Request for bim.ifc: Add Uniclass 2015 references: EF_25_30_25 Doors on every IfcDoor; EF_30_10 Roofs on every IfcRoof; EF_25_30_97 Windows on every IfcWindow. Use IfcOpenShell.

First a look at what the model holds.

```python
import ifcopenshell

model = ifcopenshell.open("bim.ifc")
print(model.schema)
print("classifications:", [c.Name for c in model.by_type("IfcClassification")])
for ifc_class in ("IfcDoor", "IfcRoof", "IfcStair", "IfcWall", "IfcWindow"):
    print(ifc_class, len(model.by_type(ifc_class)))
```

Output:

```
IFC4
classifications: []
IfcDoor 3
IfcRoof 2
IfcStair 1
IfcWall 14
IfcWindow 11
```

```python
import ifcopenshell
import ifcopenshell.api.classification

model = ifcopenshell.open("bim.ifc")

system = ifcopenshell.api.classification.add_classification(model, classification="Uniclass 2015")

codes = {
    "IfcDoor": ("EF_25_30_25", "Doors"),
    "IfcRoof": ("EF_30_10", "Roofs"),
    "IfcWindow": ("EF_25_30_97", "Windows"),
}
for ifc_class, (code, name) in codes.items():
    products = model.by_type(ifc_class)
    ifcopenshell.api.classification.add_reference(
        model, products=products, classification=system, identification=code, name=name
    )
    print(code, len(products))

model.write("bim-out.ifc")
```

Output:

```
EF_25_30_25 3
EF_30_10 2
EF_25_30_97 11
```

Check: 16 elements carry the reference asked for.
